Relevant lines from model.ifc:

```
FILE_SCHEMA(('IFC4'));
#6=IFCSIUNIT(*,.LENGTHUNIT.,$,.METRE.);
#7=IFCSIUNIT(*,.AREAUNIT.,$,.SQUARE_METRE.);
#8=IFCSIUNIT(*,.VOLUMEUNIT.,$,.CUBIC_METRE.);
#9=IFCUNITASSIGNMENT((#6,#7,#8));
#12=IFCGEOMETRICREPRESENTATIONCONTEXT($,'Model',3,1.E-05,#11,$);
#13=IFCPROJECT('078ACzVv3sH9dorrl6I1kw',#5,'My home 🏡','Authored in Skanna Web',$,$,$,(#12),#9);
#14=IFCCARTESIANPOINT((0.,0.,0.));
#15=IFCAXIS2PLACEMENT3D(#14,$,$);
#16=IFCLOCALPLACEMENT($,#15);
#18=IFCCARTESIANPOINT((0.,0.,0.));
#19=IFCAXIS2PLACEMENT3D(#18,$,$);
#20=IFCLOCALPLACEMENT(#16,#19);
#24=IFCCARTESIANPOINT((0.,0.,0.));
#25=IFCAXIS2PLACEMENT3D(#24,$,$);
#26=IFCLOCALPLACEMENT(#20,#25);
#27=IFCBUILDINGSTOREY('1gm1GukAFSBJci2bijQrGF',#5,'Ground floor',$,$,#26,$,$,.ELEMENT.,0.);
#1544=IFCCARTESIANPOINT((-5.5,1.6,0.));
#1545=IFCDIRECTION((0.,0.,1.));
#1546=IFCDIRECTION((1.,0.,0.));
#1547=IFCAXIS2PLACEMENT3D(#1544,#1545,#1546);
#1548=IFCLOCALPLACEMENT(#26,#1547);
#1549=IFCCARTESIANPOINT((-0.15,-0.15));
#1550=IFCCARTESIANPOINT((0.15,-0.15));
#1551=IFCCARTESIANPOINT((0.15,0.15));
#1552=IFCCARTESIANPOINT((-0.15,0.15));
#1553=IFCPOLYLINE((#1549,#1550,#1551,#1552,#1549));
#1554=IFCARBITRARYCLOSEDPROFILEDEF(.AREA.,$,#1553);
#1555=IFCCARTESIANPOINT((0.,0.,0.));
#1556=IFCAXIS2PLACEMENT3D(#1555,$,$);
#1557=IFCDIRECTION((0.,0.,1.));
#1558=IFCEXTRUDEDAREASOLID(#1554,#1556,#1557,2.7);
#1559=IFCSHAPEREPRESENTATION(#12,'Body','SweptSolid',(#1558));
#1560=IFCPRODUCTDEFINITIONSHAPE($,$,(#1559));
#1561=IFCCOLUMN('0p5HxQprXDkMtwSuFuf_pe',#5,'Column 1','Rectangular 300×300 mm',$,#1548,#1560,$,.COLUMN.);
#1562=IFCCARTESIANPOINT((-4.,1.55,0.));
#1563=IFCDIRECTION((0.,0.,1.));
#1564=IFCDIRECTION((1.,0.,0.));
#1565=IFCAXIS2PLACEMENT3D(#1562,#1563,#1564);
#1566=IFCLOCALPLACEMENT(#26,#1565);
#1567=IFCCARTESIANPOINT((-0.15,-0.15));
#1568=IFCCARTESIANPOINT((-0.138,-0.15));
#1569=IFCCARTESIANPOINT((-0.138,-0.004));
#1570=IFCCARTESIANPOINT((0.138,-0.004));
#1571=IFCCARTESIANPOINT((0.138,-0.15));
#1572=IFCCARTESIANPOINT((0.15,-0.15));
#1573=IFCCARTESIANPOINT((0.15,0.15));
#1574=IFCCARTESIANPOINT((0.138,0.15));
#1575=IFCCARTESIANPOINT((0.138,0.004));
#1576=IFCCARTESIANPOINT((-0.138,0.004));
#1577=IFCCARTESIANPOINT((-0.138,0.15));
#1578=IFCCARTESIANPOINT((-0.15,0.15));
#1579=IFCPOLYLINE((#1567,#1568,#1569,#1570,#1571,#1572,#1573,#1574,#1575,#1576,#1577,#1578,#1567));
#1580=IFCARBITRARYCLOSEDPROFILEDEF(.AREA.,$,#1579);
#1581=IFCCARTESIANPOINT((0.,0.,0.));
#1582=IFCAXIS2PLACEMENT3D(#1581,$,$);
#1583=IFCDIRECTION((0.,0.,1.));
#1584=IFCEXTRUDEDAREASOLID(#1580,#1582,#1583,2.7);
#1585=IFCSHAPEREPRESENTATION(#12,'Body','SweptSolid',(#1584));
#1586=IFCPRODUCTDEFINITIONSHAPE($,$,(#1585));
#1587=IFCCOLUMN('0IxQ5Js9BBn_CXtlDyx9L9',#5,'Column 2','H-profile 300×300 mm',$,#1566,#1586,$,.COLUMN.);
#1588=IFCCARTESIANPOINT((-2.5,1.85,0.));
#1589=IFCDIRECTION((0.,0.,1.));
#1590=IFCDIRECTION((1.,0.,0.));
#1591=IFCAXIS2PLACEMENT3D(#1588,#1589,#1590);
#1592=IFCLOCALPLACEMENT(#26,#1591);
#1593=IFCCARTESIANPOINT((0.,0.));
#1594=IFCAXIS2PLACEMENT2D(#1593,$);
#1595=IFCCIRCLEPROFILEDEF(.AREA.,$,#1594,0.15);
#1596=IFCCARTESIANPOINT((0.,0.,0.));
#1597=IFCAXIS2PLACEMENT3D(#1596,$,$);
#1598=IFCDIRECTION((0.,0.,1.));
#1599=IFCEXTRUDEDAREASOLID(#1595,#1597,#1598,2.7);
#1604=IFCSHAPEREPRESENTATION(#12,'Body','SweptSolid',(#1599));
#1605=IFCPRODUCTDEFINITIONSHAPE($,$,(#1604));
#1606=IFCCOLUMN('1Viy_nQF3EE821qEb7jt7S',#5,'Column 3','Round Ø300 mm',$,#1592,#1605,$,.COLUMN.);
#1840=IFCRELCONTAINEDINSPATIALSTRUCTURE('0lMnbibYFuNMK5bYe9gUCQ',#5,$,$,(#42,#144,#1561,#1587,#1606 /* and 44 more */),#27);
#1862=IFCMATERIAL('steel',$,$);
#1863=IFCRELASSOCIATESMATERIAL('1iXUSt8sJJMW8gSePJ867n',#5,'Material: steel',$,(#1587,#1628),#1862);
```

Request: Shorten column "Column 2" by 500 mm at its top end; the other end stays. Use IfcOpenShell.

```python
import ifcopenshell

model = ifcopenshell.open("model.ifc")

member = model.by_id(1587)
change = -0.5

# The extrusion runs towards the end named, so only its depth changes.
body = next(r for r in member.Representation.Representations if r.RepresentationIdentifier == "Body")
solid = body.Items[0]
old_length = solid.Depth
solid.Depth += change

print(f"length {old_length:g} -> {solid.Depth:g}")

model.write("model_rev.ifc")
```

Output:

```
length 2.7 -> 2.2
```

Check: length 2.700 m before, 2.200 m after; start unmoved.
